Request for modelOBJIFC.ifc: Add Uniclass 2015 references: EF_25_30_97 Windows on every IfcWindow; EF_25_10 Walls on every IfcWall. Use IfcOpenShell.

First a look at what the model holds.

```python
import ifcopenshell

model = ifcopenshell.open("modelOBJIFC.ifc")
print(model.schema)
print("classifications:", [c.Name for c in model.by_type("IfcClassification")])
for ifc_class in ("IfcDoor", "IfcRoof", "IfcStair", "IfcWall", "IfcWindow"):
    print(ifc_class, len(model.by_type(ifc_class)))
```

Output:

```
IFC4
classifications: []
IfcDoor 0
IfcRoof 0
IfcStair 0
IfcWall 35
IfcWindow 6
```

```python
import ifcopenshell
import ifcopenshell.api.classification

model = ifcopenshell.open("modelOBJIFC.ifc")

system = ifcopenshell.api.classification.add_classification(model, classification="Uniclass 2015")

codes = {
    "IfcWindow": ("EF_25_30_97", "Windows"),
    "IfcWall": ("EF_25_10", "Walls"),
}
for ifc_class, (code, name) in codes.items():
    products = model.by_type(ifc_class)
    ifcopenshell.api.classification.add_reference(
        model, products=products, classification=system, identification=code, name=name
    )
    print(code, len(products))

model.write("modelOBJIFC_v2.ifc")
```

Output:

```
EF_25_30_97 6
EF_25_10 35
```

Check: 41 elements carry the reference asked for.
